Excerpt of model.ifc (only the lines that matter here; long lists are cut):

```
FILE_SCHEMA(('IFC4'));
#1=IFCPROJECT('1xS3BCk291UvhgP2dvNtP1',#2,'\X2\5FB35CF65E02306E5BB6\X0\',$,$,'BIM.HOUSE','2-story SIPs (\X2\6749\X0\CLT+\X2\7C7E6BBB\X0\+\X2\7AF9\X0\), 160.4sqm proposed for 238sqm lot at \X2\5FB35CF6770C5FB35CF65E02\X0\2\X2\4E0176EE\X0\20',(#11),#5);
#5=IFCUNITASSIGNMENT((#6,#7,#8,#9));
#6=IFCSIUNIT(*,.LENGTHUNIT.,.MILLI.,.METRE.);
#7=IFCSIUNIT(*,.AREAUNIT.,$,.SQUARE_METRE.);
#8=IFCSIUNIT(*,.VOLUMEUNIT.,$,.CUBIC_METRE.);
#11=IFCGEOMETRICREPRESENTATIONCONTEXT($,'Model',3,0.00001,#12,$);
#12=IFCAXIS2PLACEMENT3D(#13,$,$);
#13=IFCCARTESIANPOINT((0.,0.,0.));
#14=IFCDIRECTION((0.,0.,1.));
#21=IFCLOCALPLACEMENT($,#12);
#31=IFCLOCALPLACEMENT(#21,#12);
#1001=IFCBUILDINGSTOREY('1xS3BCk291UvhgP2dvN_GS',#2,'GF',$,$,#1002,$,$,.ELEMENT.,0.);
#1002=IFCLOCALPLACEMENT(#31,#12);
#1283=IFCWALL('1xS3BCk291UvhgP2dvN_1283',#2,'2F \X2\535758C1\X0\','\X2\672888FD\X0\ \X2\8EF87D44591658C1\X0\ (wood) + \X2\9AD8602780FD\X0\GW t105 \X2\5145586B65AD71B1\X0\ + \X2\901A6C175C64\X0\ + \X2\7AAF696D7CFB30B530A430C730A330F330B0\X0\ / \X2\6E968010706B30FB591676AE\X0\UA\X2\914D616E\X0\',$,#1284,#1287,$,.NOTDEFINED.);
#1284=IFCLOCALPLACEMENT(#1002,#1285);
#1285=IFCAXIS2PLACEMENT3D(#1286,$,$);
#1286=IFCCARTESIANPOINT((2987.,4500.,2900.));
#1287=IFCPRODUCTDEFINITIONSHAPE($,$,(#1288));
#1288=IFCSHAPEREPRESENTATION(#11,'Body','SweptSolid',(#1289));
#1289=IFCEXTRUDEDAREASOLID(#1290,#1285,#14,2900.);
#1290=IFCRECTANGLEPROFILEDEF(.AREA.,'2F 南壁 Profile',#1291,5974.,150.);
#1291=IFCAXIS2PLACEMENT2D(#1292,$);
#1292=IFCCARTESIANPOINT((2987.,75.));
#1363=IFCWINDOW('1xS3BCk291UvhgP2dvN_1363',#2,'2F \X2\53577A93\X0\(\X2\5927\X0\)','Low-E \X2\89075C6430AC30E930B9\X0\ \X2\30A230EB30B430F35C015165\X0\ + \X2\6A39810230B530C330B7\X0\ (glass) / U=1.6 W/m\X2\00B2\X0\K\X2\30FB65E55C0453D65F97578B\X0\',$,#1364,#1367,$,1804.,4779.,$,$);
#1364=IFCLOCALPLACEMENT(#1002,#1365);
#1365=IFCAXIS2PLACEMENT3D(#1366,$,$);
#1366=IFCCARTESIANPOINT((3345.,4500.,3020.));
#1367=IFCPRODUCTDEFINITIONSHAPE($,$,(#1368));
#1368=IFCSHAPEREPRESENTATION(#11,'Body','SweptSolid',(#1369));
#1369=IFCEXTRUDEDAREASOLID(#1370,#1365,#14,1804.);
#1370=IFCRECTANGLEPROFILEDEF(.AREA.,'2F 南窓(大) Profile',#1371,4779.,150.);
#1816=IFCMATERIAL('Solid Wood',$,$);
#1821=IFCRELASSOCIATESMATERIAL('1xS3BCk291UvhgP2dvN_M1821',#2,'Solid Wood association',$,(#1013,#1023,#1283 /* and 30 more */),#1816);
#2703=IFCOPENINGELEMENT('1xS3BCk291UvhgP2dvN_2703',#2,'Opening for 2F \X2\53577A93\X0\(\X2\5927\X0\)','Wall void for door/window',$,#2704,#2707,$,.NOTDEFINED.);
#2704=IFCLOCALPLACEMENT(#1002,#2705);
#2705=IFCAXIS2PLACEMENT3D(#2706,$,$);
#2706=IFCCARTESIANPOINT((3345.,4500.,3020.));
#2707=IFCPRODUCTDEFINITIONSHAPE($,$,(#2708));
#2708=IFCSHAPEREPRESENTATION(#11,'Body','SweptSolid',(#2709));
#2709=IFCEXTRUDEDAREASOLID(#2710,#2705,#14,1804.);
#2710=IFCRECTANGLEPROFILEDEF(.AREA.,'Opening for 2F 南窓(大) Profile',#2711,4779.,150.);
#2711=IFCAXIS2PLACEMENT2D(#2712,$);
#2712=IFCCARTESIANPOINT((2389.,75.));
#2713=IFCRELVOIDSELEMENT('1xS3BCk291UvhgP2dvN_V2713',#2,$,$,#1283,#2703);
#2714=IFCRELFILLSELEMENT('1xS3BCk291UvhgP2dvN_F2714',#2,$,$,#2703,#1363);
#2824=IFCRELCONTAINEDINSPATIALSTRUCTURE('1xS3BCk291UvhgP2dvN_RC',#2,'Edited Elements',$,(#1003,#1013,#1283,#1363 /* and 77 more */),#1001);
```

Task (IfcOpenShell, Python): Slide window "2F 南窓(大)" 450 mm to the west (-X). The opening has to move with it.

```python
import ifcopenshell
import ifcopenshell.api.geometry
import ifcopenshell.util.placement

model = ifcopenshell.open("model.ifc")

window = model.by_guid("1xS3BCk291UvhgP2dvN_1363")
opening = window.FillsVoids[0].RelatingOpeningElement
wall = opening.VoidsElements[0].RelatingBuildingElement

wall_matrix = ifcopenshell.util.placement.get_local_placement(wall.ObjectPlacement)
shift = wall_matrix[:3, 0] * -450.0
before = ifcopenshell.util.placement.get_local_placement(window.ObjectPlacement)[:3, 3].copy()

# The window is not placed relative to its opening, so move both.
for product in (opening, window):
    matrix = ifcopenshell.util.placement.get_local_placement(product.ObjectPlacement)
    matrix[:3, 3] += shift
    ifcopenshell.api.geometry.edit_object_placement(model, product=product, matrix=matrix, is_si=False)

after = ifcopenshell.util.placement.get_local_placement(window.ObjectPlacement)[:3, 3]
print("window moved by", (after - before).round(3) + 0.0)

model.write("model_updated.ifc")
```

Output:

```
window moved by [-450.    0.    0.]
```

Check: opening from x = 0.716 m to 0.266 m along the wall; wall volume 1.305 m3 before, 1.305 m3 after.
